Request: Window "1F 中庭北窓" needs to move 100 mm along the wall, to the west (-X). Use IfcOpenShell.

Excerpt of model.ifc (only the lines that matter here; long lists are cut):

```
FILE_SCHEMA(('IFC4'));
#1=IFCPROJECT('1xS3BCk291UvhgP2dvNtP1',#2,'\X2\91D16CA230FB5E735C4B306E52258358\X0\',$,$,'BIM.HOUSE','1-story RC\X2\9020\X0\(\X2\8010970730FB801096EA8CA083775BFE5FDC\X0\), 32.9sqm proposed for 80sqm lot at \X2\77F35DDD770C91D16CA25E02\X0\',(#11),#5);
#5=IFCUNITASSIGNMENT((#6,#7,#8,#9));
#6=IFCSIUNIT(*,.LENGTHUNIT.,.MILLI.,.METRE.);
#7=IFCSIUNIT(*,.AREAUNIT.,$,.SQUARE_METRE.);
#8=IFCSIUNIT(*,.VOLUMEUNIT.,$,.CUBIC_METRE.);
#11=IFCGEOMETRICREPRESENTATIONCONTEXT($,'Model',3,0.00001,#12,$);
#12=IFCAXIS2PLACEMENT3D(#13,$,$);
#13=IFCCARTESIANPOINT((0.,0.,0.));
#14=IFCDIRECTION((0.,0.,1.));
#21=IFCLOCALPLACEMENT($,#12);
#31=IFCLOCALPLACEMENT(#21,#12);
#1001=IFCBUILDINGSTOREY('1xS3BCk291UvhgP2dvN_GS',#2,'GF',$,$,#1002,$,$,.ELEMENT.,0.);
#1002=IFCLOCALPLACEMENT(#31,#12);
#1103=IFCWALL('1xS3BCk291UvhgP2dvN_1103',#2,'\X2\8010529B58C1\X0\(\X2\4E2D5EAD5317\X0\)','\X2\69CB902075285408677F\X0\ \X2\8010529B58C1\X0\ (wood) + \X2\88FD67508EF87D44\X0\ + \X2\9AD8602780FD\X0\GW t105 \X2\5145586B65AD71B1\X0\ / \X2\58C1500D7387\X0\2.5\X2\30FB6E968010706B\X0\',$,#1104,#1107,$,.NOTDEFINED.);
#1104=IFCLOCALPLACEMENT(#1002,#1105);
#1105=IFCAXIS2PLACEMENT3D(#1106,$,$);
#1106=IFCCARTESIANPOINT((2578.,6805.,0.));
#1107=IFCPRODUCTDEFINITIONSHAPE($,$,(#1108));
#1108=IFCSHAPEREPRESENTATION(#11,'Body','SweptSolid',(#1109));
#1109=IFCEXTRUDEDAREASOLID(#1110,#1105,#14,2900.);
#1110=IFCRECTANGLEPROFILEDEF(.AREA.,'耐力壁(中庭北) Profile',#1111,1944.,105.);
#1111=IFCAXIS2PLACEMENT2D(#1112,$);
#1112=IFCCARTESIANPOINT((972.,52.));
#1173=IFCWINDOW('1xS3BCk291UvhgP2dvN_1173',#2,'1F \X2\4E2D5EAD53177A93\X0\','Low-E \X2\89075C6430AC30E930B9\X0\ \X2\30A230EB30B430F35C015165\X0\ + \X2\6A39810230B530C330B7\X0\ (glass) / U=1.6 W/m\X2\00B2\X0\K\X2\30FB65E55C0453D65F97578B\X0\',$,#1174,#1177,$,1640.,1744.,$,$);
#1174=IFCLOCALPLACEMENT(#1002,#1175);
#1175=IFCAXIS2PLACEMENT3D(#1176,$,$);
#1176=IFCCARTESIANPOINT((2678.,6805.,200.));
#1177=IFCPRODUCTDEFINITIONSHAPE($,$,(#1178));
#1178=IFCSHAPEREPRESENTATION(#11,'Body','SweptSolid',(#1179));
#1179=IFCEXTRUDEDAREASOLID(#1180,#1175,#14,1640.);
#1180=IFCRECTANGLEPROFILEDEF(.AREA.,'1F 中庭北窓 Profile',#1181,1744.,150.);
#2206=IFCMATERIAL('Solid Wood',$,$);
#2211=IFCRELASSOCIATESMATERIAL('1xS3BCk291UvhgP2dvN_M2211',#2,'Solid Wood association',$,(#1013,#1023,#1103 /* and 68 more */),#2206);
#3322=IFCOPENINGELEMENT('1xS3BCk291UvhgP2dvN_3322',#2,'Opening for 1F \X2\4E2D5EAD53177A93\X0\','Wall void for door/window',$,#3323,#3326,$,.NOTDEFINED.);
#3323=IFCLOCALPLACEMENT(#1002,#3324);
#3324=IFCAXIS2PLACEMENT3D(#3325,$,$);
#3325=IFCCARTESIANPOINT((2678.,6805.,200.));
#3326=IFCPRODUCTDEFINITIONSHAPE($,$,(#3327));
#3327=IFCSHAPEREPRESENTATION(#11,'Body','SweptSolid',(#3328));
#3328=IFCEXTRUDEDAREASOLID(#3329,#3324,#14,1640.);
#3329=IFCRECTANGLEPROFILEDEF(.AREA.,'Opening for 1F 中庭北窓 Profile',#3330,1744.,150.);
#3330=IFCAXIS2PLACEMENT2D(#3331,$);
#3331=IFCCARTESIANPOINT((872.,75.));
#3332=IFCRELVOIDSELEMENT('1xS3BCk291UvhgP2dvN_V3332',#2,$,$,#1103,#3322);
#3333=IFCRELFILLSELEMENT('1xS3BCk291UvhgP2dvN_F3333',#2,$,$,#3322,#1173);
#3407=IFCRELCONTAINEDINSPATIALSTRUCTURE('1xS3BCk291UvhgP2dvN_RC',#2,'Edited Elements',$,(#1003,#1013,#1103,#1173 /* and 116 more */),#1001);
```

```python
import ifcopenshell
import ifcopenshell.api.geometry
import ifcopenshell.util.placement
import ifcopenshell.util.unit

model = ifcopenshell.open("model.ifc")
unit_scale = ifcopenshell.util.unit.calculate_unit_scale(model)

window = model.by_guid("1xS3BCk291UvhgP2dvN_1173")
opening = window.FillsVoids[0].RelatingOpeningElement
wall = opening.VoidsElements[0].RelatingBuildingElement

wall_matrix = ifcopenshell.util.placement.get_local_placement(wall.ObjectPlacement)
shift = wall_matrix[:3, 0] * -0.1 / unit_scale
before = ifcopenshell.util.placement.get_local_placement(window.ObjectPlacement)[:3, 3].copy()

# The window is not placed relative to its opening, so move both.
for product in (opening, window):
    matrix = ifcopenshell.util.placement.get_local_placement(product.ObjectPlacement)
    matrix[:3, 3] += shift
    ifcopenshell.api.geometry.edit_object_placement(model, product=product, matrix=matrix, is_si=False)

after = ifcopenshell.util.placement.get_local_placement(window.ObjectPlacement)[:3, 3]
print("window moved by", (after - before).round(3) + 0.0)

model.write("model-out.ifc")
```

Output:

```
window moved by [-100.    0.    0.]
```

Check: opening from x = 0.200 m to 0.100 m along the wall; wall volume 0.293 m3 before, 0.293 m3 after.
